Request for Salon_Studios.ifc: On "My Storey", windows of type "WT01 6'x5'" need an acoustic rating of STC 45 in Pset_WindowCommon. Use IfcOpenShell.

First a look at what the model holds.

```python
import ifcopenshell
import ifcopenshell.util.element

model = ifcopenshell.open("Salon_Studios.ifc")
print(model.schema)
storey = next(s for s in model.by_type("IfcBuildingStorey") if s.Name == "My Storey")
windows = [e for e in ifcopenshell.util.element.get_decomposition(storey) if e.is_a("IfcWindow")]
seen = {}
for e in windows:
    element_type = ifcopenshell.util.element.get_type(e)
    key = (element_type.Name if element_type != e and element_type else None, ifcopenshell.util.element.get_pset(e, "Pset_WindowCommon", "AcousticRating"))
    seen[key] = seen.get(key, 0) + 1
for (name, value), count in sorted(seen.items(), key=str):
    print(count, "x", name, "|", value)
```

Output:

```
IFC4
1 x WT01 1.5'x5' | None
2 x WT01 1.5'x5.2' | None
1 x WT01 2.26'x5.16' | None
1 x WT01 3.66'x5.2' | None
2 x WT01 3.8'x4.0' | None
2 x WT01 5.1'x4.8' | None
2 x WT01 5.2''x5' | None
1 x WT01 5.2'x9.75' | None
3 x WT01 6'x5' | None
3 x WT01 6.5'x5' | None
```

```python
import ifcopenshell
import ifcopenshell.api.pset
import ifcopenshell.util.element

model = ifcopenshell.open("Salon_Studios.ifc")

storey = next(s for s in model.by_type("IfcBuildingStorey") if s.Name == "My Storey")
windows = [e for e in ifcopenshell.util.element.get_decomposition(storey) if e.is_a("IfcWindow")]

count = 0
for e in windows:
    element_type = ifcopenshell.util.element.get_type(e)
    if element_type in (None, e) or element_type.Name != "WT01 6'x5'":
        continue
    # add_pset returns the element's existing set when there is one.
    pset = ifcopenshell.api.pset.add_pset(model, product=e, name="Pset_WindowCommon")
    ifcopenshell.api.pset.edit_pset(model, pset=pset, properties={"AcousticRating": "STC 45"})
    count += 1

print(count, "windows updated")

model.write("Salon_Studios_updated.ifc")
```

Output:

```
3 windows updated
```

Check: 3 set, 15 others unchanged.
